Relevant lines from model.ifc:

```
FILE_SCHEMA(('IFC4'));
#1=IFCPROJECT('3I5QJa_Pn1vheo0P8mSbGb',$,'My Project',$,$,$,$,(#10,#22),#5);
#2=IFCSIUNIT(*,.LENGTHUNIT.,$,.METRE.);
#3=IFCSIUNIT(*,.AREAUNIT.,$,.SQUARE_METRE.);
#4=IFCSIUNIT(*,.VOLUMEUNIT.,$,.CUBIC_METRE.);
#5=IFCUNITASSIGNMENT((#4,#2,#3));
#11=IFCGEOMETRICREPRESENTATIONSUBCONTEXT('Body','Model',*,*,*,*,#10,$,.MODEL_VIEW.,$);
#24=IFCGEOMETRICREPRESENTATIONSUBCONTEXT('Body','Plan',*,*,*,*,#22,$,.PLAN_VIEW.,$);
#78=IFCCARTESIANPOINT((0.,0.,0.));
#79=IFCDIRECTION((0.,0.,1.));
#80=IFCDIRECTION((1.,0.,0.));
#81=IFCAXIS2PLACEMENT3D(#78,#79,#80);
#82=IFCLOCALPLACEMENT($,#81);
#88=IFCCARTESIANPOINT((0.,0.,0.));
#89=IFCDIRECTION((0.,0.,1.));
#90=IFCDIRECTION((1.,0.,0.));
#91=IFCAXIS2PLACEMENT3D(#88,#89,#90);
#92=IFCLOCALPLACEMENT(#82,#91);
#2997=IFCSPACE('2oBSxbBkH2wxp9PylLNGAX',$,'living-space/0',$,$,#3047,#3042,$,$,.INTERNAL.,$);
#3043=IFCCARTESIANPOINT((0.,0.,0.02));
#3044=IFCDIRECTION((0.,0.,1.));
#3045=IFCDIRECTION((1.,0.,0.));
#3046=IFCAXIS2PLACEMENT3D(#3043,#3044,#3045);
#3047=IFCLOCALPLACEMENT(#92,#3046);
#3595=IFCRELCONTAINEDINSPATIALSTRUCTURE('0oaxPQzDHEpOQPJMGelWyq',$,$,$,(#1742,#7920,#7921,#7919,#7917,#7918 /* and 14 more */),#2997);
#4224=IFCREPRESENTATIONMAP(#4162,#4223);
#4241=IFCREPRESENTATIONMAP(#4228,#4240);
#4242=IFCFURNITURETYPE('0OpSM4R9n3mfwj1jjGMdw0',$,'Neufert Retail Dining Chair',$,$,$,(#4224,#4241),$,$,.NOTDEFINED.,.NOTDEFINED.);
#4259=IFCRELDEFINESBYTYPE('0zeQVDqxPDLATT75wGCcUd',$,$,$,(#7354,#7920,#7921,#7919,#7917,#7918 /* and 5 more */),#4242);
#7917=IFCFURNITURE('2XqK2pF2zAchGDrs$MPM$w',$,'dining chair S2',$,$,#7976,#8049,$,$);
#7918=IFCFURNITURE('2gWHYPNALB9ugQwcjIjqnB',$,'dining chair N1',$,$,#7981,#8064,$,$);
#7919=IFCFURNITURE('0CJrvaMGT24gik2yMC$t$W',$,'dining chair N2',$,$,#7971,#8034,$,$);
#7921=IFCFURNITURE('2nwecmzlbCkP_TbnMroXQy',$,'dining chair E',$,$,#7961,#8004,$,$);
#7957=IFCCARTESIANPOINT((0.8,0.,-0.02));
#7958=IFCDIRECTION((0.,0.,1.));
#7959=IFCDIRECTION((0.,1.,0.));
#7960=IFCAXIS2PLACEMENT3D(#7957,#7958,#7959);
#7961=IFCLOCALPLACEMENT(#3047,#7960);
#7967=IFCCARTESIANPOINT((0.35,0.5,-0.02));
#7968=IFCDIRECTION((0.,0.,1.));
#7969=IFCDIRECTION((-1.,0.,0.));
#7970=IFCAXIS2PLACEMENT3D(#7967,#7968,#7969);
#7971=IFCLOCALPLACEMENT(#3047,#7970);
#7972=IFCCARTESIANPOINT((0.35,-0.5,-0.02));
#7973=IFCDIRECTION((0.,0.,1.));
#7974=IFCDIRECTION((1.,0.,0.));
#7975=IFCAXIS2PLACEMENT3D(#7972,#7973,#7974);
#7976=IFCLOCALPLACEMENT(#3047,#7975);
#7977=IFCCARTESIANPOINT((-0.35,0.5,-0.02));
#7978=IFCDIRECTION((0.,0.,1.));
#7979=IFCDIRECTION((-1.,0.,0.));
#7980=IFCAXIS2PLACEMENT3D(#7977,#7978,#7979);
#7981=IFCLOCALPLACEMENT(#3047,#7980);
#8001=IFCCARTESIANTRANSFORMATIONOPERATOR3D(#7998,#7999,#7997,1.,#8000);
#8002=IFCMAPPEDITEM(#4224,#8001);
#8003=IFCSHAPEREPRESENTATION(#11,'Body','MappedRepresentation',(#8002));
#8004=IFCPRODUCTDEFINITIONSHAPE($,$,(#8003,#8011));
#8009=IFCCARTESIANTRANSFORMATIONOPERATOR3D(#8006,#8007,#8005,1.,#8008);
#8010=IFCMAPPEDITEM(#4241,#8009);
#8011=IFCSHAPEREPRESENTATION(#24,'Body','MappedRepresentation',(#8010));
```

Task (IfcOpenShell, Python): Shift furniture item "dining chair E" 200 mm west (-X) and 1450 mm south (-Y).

```python
import ifcopenshell
import ifcopenshell.api.geometry
import ifcopenshell.util.placement

model = ifcopenshell.open("model.ifc")

item = model.by_id(7921)
matrix = ifcopenshell.util.placement.get_local_placement(item.ObjectPlacement)
matrix[0, 3] -= 0.2
matrix[1, 3] -= 1.45
ifcopenshell.api.geometry.edit_object_placement(model, product=item, matrix=matrix, is_si=False)

print(ifcopenshell.util.placement.get_local_placement(item.ObjectPlacement).round(3) + 0.0)

model.write("model_edited.ifc")
```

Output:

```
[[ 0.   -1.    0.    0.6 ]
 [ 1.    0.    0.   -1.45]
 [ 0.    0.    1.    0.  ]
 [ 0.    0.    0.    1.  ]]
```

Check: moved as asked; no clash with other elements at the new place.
